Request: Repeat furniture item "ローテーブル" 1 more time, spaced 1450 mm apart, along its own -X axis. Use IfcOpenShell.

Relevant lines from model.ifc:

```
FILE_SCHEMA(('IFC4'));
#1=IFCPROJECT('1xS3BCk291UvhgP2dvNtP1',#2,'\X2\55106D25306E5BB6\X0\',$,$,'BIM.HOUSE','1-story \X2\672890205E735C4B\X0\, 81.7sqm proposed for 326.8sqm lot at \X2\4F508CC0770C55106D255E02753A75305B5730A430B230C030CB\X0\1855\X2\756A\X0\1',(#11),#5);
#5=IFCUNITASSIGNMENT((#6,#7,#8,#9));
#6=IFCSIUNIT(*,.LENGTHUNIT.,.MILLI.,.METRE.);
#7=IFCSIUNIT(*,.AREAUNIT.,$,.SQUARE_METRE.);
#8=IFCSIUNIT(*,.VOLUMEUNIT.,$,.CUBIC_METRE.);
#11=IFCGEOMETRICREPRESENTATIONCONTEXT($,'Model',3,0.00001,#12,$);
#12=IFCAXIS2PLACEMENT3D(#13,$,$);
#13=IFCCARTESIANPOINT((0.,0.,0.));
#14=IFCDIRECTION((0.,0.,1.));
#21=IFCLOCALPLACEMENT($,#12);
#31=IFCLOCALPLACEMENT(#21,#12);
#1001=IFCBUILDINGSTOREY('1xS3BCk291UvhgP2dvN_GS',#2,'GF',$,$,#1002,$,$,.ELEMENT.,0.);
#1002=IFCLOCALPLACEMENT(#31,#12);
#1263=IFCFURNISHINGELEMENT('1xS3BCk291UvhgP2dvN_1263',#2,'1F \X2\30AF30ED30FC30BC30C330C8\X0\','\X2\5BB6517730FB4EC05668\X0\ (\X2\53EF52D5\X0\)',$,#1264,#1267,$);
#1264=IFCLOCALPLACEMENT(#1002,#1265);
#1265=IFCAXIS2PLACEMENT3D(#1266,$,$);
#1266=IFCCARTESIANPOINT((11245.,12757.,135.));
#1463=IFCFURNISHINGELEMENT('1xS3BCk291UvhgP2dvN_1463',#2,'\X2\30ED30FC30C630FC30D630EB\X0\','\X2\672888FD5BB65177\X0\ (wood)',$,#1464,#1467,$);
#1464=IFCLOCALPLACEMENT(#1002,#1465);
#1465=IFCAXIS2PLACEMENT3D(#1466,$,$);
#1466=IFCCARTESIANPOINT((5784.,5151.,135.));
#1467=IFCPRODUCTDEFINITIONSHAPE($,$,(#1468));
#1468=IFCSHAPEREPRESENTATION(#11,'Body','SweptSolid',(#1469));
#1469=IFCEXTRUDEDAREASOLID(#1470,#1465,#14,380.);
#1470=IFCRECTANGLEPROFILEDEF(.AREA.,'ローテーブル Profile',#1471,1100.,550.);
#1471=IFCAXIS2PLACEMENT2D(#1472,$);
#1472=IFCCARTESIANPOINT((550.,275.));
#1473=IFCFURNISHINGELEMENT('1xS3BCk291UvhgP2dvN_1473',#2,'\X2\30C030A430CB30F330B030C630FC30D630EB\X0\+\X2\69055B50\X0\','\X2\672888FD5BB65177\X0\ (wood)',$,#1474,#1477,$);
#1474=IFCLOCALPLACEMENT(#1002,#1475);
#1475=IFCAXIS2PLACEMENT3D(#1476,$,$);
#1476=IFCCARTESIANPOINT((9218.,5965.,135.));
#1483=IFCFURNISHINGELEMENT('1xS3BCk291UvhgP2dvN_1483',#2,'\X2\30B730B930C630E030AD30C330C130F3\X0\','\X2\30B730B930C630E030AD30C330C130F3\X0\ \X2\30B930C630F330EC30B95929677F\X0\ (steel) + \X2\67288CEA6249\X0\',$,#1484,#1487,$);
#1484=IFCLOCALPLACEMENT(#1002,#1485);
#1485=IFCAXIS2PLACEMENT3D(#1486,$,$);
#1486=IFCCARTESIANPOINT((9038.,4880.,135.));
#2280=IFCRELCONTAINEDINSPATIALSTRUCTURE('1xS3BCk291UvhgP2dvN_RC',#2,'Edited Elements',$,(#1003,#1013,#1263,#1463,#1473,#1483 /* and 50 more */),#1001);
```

```python
import ifcopenshell
import ifcopenshell.api.geometry
import ifcopenshell.api.root
import ifcopenshell.util.element
import ifcopenshell.util.placement
import ifcopenshell.util.unit

model = ifcopenshell.open("model.ifc")
unit_scale = ifcopenshell.util.unit.calculate_unit_scale(model)


def reuse_history(source, copy):
    """copy_class also copies each property set's owner history, people and application; keep the originals."""
    for rel in copy.IsDefinedBy:
        if rel.is_a("IfcRelDefinesByProperties") and (history := rel.RelatingPropertyDefinition.OwnerHistory):
            rel.RelatingPropertyDefinition.OwnerHistory = source.OwnerHistory
            ifcopenshell.util.element.remove_deep2(model, history)


source = model.by_guid("1xS3BCk291UvhgP2dvN_1463")
base = ifcopenshell.util.placement.get_local_placement(source.ObjectPlacement)
step = -base[:3, 0] * 1.45 / unit_scale

for i in range(1, 2):
    copy = ifcopenshell.api.root.copy_class(model, product=source)
    copy.Representation = ifcopenshell.util.element.copy_deep(
        model, source.Representation, exclude=["IfcGeometricRepresentationContext", "IfcRepresentationMap"]
    )
    reuse_history(source, copy)
    matrix = base.copy()
    matrix[:3, 3] += i * step
    print("added at", matrix[:3, 3].round(3) + 0.0)
    ifcopenshell.api.geometry.edit_object_placement(model, product=copy, matrix=matrix, is_si=False)

model.write("model-out.ifc")
```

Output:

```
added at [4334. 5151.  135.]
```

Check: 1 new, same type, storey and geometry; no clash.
